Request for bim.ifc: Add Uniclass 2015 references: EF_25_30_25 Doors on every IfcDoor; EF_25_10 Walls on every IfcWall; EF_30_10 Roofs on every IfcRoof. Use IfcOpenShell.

First a look at what the model holds.

```python
import ifcopenshell

model = ifcopenshell.open("bim.ifc")
print(model.schema)
print("classifications:", [c.Name for c in model.by_type("IfcClassification")])
for ifc_class in ("IfcDoor", "IfcRoof", "IfcStair", "IfcWall", "IfcWindow"):
    print(ifc_class, len(model.by_type(ifc_class)))
```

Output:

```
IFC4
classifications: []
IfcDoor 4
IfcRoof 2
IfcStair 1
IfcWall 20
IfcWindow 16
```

```python
import ifcopenshell
import ifcopenshell.api.classification

model = ifcopenshell.open("bim.ifc")

system = ifcopenshell.api.classification.add_classification(model, classification="Uniclass 2015")

codes = {
    "IfcDoor": ("EF_25_30_25", "Doors"),
    "IfcWall": ("EF_25_10", "Walls"),
    "IfcRoof": ("EF_30_10", "Roofs"),
}
for ifc_class, (code, name) in codes.items():
    products = model.by_type(ifc_class)
    ifcopenshell.api.classification.add_reference(
        model, products=products, classification=system, identification=code, name=name
    )
    print(code, len(products))

model.write("bim_updated.ifc")
```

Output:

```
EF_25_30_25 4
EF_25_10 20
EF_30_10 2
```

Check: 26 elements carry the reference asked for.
